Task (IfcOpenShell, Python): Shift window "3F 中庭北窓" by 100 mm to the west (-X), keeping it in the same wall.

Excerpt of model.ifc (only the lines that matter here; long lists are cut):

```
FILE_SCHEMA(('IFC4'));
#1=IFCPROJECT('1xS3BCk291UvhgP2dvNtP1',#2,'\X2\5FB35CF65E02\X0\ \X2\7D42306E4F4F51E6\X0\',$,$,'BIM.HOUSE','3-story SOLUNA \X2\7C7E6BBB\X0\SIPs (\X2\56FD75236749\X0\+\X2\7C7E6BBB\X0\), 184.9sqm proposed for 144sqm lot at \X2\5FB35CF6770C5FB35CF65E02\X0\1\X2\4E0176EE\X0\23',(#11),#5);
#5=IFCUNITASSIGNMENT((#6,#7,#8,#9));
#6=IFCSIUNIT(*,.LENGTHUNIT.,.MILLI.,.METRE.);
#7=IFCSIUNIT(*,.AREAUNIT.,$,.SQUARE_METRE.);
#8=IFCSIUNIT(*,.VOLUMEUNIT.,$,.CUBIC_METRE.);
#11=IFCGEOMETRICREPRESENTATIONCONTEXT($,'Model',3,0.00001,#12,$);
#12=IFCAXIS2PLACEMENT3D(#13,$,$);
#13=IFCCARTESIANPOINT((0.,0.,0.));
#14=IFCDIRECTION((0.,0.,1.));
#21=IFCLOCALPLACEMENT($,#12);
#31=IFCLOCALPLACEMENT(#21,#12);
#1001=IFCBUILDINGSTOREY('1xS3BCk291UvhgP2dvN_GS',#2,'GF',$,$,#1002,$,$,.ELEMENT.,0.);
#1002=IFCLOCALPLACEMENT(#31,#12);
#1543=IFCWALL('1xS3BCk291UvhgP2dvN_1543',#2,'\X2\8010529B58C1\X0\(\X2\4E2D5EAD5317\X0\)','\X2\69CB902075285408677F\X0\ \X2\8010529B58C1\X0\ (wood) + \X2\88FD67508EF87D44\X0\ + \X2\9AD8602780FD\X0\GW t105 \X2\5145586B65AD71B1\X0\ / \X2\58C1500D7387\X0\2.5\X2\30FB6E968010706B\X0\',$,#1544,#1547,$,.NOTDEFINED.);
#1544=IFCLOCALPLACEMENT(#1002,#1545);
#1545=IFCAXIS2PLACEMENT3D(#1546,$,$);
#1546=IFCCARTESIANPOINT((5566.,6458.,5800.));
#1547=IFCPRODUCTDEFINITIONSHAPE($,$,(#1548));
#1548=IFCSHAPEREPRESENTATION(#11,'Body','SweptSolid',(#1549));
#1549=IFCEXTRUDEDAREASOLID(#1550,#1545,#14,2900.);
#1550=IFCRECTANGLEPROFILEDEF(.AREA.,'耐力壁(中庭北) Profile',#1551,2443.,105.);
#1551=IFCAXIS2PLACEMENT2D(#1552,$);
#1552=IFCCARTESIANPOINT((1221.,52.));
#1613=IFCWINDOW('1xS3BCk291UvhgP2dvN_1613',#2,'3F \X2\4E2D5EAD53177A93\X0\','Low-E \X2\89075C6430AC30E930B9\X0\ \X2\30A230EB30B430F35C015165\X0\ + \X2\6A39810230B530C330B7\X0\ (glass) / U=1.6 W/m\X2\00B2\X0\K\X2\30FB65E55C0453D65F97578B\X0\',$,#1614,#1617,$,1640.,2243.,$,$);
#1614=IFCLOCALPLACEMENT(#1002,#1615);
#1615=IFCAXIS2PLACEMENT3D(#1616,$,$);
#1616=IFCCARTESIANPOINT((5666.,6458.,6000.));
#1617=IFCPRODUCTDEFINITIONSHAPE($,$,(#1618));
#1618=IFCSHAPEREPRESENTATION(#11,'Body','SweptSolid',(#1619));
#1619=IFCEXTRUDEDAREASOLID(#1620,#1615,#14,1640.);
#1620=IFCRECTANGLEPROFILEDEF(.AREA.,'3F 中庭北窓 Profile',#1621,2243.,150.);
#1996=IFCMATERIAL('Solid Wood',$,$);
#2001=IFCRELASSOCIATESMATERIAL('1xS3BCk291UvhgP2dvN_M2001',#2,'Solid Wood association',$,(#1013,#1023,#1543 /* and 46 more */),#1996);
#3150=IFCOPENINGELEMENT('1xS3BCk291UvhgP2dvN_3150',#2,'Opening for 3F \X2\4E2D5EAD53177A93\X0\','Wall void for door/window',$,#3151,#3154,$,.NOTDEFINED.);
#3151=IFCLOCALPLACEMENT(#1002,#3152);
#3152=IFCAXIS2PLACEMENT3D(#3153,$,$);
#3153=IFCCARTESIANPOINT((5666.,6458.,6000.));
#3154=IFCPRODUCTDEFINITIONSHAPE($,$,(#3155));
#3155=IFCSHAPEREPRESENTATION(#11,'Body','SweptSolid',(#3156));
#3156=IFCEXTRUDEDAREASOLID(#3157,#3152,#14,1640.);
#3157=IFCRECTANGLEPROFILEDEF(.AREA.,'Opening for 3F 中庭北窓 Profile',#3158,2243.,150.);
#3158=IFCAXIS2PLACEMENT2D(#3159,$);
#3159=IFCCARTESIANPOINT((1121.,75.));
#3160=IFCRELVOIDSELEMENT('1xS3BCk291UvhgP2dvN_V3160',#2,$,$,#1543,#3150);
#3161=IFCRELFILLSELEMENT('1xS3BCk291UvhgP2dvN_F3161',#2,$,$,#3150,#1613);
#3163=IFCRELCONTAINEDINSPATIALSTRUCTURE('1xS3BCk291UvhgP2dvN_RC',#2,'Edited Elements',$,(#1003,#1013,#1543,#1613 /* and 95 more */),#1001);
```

```python
import ifcopenshell
import ifcopenshell.api.geometry
import ifcopenshell.util.placement

model = ifcopenshell.open("model.ifc")

window = model.by_guid("1xS3BCk291UvhgP2dvN_1613")
opening = window.FillsVoids[0].RelatingOpeningElement
wall = opening.VoidsElements[0].RelatingBuildingElement

wall_matrix = ifcopenshell.util.placement.get_local_placement(wall.ObjectPlacement)
shift = wall_matrix[:3, 0] * -100.0
before = ifcopenshell.util.placement.get_local_placement(window.ObjectPlacement)[:3, 3].copy()

# The window is not placed relative to its opening, so move both.
for product in (opening, window):
    matrix = ifcopenshell.util.placement.get_local_placement(product.ObjectPlacement)
    matrix[:3, 3] += shift
    ifcopenshell.api.geometry.edit_object_placement(model, product=product, matrix=matrix, is_si=False)

after = ifcopenshell.util.placement.get_local_placement(window.ObjectPlacement)[:3, 3]
print("window moved by", (after - before).round(3) + 0.0)

model.write("model_edited.ifc")
```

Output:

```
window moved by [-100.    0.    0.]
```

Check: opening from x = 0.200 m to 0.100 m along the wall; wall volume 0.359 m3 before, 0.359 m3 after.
